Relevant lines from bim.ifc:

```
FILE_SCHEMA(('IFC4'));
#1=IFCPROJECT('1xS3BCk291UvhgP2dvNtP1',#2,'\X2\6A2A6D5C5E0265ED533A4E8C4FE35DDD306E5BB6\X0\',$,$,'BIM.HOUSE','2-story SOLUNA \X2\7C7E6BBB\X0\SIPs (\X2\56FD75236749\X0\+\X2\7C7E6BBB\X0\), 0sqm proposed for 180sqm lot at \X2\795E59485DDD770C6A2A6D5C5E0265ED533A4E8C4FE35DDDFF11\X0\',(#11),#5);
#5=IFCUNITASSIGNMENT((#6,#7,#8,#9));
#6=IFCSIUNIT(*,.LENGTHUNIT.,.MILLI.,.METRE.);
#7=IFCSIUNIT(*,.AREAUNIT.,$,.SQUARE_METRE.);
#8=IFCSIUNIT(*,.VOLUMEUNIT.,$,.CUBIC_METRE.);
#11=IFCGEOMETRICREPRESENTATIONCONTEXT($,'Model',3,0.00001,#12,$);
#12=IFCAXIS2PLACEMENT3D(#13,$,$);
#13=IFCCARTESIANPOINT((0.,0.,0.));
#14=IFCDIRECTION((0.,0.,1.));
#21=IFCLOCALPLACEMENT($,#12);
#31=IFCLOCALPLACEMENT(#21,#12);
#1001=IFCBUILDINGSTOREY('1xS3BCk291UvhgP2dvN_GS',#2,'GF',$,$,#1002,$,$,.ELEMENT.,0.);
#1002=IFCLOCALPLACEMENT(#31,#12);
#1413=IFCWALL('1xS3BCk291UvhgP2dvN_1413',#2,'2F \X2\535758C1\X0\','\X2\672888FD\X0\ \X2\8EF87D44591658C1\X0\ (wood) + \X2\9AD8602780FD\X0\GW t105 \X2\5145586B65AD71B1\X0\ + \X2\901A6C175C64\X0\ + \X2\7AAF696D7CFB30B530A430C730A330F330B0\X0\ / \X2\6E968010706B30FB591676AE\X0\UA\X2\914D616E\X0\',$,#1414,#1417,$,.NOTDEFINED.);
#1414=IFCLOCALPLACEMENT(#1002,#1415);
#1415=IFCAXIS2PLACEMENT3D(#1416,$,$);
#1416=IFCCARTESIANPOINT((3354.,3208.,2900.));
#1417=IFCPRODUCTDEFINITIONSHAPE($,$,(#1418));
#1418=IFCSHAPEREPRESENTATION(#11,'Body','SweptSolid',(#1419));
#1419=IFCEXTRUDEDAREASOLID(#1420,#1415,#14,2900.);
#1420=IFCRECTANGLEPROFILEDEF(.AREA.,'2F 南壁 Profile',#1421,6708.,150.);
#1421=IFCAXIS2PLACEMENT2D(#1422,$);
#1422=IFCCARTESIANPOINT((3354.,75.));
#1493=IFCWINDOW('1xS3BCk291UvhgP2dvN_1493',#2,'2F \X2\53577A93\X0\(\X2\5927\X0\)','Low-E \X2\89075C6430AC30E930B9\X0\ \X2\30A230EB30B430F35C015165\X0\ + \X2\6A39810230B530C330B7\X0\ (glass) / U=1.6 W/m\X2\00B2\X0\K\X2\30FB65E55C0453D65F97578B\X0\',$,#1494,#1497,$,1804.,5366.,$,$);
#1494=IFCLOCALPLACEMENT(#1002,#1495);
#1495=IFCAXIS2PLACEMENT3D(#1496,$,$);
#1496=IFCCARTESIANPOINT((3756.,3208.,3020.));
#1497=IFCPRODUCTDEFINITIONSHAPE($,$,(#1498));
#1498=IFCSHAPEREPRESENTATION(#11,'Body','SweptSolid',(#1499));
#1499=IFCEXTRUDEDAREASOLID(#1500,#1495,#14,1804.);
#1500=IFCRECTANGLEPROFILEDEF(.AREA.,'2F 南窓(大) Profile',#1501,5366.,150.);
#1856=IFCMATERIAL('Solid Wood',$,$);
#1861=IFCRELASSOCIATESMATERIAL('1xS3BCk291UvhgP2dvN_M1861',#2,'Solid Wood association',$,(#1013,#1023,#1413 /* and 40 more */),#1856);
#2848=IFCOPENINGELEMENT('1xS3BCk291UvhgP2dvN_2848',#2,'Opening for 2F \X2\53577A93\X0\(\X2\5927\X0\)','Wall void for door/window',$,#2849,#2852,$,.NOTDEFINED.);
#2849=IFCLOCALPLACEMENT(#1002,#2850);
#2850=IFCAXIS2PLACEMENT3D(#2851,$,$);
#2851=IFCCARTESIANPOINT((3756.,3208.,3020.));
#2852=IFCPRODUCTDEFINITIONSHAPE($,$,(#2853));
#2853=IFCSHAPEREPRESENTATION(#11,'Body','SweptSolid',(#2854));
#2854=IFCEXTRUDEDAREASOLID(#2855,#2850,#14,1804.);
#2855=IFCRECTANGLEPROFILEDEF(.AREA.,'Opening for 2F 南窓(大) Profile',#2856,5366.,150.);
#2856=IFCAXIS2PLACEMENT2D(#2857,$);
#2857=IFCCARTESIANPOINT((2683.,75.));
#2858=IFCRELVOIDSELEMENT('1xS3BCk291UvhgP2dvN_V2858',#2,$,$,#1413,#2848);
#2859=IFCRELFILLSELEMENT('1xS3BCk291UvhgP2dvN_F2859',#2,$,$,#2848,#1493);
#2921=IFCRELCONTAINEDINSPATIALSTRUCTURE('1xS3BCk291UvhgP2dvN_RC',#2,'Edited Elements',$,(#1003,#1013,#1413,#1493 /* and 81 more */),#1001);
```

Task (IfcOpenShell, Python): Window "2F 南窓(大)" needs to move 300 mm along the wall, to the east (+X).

```python
import ifcopenshell
import ifcopenshell.api.geometry
import ifcopenshell.util.placement
import ifcopenshell.util.unit

model = ifcopenshell.open("bim.ifc")
unit_scale = ifcopenshell.util.unit.calculate_unit_scale(model)

window = model.by_guid("1xS3BCk291UvhgP2dvN_1493")
opening = window.FillsVoids[0].RelatingOpeningElement
wall = opening.VoidsElements[0].RelatingBuildingElement

wall_matrix = ifcopenshell.util.placement.get_local_placement(wall.ObjectPlacement)
shift = wall_matrix[:3, 0] * 0.3 / unit_scale
before = ifcopenshell.util.placement.get_local_placement(window.ObjectPlacement)[:3, 3].copy()

# The window is not placed relative to its opening, so move both.
for product in (opening, window):
    matrix = ifcopenshell.util.placement.get_local_placement(product.ObjectPlacement)
    matrix[:3, 3] += shift
    ifcopenshell.api.geometry.edit_object_placement(model, product=product, matrix=matrix, is_si=False)

after = ifcopenshell.util.placement.get_local_placement(window.ObjectPlacement)[:3, 3]
print("window moved by", (after - before).round(3) + 0.0)

model.write("bim_v2.ifc")
```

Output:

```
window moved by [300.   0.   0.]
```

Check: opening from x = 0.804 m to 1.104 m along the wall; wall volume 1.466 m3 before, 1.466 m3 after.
